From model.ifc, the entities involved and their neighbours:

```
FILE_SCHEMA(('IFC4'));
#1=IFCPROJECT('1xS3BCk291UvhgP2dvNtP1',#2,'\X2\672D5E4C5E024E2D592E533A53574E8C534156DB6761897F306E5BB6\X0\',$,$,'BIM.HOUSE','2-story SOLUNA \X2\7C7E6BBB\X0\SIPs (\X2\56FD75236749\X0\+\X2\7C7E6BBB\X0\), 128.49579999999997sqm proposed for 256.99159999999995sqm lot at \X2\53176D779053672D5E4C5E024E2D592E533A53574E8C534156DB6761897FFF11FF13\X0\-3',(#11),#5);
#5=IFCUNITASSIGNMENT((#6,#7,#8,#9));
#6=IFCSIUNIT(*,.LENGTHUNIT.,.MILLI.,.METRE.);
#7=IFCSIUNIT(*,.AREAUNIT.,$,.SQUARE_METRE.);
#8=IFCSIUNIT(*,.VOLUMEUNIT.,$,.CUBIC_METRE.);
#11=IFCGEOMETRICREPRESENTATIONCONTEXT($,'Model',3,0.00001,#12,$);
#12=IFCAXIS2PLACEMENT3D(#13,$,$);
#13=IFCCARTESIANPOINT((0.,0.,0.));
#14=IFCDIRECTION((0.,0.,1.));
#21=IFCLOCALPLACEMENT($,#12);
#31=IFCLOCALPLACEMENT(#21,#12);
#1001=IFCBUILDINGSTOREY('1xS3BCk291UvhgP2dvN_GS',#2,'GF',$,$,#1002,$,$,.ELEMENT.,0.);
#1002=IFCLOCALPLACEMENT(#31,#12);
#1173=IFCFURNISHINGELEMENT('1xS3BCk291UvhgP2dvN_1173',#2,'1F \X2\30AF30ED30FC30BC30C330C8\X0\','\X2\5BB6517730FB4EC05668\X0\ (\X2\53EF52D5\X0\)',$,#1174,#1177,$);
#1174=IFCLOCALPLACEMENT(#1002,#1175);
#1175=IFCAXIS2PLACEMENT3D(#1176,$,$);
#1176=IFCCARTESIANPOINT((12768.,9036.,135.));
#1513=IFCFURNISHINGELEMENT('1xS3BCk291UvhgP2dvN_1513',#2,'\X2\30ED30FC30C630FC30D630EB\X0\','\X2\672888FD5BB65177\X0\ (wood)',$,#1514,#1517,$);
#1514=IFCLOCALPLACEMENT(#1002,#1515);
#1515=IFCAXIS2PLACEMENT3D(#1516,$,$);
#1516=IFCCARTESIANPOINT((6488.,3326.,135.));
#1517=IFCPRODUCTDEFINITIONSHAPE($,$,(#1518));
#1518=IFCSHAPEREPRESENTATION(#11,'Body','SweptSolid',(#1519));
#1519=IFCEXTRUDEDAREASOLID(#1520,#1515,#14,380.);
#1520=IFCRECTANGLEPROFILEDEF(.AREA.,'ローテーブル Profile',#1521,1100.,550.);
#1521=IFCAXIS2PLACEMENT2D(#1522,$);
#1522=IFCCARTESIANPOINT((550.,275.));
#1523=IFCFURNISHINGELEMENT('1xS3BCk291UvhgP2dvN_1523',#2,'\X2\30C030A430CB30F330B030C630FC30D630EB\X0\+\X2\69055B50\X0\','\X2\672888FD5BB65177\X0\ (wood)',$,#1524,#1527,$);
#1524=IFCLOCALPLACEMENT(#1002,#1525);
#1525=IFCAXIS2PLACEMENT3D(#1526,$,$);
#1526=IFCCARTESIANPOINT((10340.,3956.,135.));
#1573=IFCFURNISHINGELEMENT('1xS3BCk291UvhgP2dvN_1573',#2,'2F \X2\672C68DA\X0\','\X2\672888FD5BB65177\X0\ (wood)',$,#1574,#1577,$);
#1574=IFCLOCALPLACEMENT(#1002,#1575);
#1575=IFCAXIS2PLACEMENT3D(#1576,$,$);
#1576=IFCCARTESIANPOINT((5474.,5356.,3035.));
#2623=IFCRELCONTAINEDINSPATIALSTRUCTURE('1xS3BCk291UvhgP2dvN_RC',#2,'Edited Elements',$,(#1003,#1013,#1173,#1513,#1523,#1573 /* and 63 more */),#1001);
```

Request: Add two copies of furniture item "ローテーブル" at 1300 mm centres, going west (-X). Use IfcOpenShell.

```python
import numpy as np
import ifcopenshell
import ifcopenshell.api.geometry
import ifcopenshell.api.root
import ifcopenshell.util.element
import ifcopenshell.util.placement

model = ifcopenshell.open("model.ifc")


def reuse_history(source, copy):
    """copy_class also copies each property set's owner history, people and application; keep the originals."""
    for rel in copy.IsDefinedBy:
        if rel.is_a("IfcRelDefinesByProperties") and (history := rel.RelatingPropertyDefinition.OwnerHistory):
            rel.RelatingPropertyDefinition.OwnerHistory = source.OwnerHistory
            ifcopenshell.util.element.remove_deep2(model, history)


source = model.by_guid("1xS3BCk291UvhgP2dvN_1513")
base = ifcopenshell.util.placement.get_local_placement(source.ObjectPlacement)
step = np.array([-1.0, 0.0, 0.0]) * 1300.0

for i in range(1, 3):
    copy = ifcopenshell.api.root.copy_class(model, product=source)
    copy.Representation = ifcopenshell.util.element.copy_deep(
        model, source.Representation, exclude=["IfcGeometricRepresentationContext", "IfcRepresentationMap"]
    )
    reuse_history(source, copy)
    matrix = base.copy()
    matrix[:3, 3] += i * step
    print("added at", matrix[:3, 3].round(3) + 0.0)
    ifcopenshell.api.geometry.edit_object_placement(model, product=copy, matrix=matrix, is_si=False)

model.write("model_v2.ifc")
```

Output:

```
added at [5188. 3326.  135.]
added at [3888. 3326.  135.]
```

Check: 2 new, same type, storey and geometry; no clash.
